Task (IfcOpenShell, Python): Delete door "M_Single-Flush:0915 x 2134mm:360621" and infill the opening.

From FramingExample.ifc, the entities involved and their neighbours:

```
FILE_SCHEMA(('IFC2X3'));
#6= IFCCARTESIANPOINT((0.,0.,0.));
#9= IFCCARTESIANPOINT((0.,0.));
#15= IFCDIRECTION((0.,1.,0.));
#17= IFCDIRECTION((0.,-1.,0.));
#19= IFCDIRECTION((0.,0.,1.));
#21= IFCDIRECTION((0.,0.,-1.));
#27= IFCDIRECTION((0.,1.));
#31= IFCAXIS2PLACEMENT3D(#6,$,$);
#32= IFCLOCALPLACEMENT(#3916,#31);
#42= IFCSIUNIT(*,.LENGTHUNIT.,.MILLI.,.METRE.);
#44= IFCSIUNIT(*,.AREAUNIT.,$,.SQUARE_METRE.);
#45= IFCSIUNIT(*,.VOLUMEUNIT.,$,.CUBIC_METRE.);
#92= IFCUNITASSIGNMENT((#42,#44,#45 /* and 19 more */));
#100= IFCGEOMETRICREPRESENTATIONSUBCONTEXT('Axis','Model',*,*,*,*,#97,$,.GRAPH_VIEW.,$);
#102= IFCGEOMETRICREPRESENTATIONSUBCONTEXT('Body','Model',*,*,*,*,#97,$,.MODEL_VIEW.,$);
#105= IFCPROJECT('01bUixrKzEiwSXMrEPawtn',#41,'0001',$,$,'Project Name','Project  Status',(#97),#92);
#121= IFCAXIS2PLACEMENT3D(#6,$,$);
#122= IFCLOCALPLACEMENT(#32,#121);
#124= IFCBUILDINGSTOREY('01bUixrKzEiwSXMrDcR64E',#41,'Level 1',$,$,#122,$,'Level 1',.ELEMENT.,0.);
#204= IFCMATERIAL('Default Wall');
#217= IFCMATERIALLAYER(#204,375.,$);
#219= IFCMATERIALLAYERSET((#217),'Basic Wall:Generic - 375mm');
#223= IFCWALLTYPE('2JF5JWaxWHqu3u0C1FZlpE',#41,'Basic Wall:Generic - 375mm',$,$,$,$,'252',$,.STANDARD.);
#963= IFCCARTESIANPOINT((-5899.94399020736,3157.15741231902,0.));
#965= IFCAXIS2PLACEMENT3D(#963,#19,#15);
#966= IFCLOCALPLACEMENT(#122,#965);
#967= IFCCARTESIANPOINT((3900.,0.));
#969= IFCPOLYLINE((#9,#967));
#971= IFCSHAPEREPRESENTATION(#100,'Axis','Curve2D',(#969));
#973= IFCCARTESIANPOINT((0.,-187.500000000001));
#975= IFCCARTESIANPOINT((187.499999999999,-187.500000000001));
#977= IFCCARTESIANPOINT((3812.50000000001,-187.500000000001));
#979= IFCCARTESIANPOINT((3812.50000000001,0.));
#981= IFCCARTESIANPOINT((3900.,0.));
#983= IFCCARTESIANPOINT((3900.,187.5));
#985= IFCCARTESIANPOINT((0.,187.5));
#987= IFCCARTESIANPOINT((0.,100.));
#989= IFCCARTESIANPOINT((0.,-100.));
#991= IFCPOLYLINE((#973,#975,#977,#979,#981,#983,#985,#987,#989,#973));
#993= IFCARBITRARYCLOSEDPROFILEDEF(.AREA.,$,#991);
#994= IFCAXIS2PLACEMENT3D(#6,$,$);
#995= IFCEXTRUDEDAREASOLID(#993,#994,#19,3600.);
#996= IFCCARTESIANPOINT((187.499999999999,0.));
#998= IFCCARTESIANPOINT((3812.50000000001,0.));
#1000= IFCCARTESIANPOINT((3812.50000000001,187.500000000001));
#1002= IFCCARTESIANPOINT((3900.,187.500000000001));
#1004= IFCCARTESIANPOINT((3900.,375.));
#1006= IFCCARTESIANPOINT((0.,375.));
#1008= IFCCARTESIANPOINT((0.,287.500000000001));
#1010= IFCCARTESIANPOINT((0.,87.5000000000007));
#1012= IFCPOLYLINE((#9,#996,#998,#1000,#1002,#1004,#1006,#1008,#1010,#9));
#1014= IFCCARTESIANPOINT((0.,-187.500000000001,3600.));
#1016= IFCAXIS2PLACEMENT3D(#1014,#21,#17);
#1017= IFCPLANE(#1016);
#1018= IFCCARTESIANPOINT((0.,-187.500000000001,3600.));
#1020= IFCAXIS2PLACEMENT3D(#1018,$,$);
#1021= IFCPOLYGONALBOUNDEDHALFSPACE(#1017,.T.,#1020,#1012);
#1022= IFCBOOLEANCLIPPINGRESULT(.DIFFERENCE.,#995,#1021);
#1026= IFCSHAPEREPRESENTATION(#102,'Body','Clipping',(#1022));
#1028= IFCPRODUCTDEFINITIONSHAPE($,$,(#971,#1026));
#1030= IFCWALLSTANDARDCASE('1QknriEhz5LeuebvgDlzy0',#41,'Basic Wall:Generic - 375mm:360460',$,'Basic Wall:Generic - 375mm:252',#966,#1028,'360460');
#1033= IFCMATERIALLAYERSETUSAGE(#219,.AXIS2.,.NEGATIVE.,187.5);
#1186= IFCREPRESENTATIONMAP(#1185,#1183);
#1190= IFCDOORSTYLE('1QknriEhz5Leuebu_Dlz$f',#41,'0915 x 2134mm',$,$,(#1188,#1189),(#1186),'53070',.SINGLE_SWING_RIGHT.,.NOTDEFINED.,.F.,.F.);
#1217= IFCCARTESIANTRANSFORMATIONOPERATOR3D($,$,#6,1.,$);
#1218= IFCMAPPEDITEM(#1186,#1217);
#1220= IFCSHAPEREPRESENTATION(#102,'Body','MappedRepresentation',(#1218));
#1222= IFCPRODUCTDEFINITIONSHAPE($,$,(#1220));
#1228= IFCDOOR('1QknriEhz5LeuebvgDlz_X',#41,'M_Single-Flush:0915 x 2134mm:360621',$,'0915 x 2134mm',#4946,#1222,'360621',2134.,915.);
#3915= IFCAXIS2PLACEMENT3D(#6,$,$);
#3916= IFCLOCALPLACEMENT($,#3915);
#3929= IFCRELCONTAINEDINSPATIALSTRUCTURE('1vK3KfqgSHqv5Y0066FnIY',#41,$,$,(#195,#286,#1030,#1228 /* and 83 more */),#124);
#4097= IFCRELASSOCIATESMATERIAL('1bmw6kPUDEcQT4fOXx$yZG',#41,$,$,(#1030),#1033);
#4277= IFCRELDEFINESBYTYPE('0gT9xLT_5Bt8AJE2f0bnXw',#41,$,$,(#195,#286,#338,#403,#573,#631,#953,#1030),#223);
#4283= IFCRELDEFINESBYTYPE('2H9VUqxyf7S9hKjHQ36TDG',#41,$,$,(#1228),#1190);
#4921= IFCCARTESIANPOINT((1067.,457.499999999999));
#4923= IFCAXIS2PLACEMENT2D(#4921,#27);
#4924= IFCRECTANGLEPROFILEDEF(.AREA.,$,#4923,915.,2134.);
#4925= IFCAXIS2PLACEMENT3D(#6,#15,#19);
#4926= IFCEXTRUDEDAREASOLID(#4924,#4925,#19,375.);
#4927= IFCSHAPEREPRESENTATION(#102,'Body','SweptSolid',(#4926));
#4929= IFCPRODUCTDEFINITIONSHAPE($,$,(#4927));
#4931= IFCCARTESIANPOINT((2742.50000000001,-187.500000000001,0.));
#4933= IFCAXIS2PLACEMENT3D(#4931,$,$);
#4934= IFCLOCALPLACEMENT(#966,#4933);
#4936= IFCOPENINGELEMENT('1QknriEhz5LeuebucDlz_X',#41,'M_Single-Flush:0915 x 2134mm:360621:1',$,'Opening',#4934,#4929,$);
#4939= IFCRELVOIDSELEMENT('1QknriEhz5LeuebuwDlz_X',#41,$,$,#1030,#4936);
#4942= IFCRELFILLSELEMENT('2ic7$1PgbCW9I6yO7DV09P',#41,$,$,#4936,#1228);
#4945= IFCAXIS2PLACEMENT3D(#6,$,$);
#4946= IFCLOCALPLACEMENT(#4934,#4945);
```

```python
import ifcopenshell
import ifcopenshell.api.feature
import ifcopenshell.api.root
import ifcopenshell.geom
import ifcopenshell.util.shape

model = ifcopenshell.open("FramingExample.ifc")
settings = ifcopenshell.geom.settings()


def volume(element):
    """Net volume in cubic metres, openings subtracted."""
    shape = ifcopenshell.geom.create_shape(settings, element)
    return ifcopenshell.util.shape.get_volume(shape.geometry)


door = model.by_id(1228)
opening = door.FillsVoids[0].RelatingOpeningElement
wall = opening.VoidsElements[0].RelatingBuildingElement
before = volume(wall)

ifcopenshell.api.root.remove_product(model, product=door)
ifcopenshell.api.feature.remove_feature(model, feature=opening)

after = volume(wall)

print(f"wall volume {before:.3f} -> {after:.3f} m3")

model.write("FramingExample_updated.ifc")
```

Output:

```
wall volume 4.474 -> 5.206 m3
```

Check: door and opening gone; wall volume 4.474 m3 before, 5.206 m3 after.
